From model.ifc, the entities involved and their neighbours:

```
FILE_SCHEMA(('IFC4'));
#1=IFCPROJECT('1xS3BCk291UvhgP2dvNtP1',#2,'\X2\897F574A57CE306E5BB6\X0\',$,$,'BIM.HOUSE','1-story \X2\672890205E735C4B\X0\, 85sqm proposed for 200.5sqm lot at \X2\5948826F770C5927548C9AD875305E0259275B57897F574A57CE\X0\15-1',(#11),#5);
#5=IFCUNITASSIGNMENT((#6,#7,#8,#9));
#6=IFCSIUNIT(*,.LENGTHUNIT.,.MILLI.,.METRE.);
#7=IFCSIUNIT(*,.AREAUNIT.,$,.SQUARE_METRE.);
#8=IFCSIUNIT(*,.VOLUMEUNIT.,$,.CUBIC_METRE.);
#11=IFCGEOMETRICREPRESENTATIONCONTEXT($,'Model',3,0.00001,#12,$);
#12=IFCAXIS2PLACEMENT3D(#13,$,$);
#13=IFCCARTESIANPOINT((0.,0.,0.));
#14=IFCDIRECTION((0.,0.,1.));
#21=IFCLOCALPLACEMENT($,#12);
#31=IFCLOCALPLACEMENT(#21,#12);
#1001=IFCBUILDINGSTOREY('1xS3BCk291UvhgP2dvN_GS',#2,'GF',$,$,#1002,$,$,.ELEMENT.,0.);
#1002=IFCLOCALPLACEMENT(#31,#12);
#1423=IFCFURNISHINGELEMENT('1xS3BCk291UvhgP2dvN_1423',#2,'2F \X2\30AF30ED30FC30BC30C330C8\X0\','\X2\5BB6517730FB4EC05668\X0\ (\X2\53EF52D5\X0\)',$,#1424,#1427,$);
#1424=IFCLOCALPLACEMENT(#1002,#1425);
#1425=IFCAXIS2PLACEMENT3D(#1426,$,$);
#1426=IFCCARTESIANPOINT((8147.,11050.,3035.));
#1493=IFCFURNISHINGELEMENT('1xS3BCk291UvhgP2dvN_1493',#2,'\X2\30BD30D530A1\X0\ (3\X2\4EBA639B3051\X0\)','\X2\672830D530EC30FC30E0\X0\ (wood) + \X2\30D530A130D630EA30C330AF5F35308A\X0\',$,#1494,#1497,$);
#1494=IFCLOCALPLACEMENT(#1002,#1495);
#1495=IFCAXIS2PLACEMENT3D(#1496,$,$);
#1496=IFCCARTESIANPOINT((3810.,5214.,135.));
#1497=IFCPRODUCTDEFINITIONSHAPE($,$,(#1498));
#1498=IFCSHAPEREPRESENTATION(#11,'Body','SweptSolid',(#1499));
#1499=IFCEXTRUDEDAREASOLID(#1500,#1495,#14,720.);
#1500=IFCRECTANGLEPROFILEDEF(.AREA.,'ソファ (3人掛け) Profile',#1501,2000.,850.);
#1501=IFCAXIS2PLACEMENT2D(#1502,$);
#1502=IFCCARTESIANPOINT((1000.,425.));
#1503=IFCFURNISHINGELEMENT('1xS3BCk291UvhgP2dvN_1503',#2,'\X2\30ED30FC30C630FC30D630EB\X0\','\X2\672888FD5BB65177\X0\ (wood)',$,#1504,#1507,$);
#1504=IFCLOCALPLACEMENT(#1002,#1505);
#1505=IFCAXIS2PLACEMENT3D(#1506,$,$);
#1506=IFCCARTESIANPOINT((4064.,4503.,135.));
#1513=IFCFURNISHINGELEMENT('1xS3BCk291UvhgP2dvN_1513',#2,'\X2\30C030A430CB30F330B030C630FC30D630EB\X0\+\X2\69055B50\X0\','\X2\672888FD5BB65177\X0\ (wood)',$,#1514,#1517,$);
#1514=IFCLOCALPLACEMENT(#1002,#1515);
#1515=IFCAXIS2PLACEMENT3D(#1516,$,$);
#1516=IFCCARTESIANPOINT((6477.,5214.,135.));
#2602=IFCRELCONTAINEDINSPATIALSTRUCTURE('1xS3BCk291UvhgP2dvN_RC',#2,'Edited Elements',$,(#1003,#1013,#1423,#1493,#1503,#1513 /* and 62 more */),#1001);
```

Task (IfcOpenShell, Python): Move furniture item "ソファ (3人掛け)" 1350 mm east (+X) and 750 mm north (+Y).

```python
import ifcopenshell
import ifcopenshell.api.geometry
import ifcopenshell.util.placement
import ifcopenshell.util.unit

model = ifcopenshell.open("model.ifc")
unit_scale = ifcopenshell.util.unit.calculate_unit_scale(model)

item = model.by_guid("1xS3BCk291UvhgP2dvN_1493")
matrix = ifcopenshell.util.placement.get_local_placement(item.ObjectPlacement)
matrix[0, 3] += 1.35 / unit_scale
matrix[1, 3] += 0.75 / unit_scale
ifcopenshell.api.geometry.edit_object_placement(model, product=item, matrix=matrix, is_si=False)

print(ifcopenshell.util.placement.get_local_placement(item.ObjectPlacement).round(3) + 0.0)

model.write("model_rev.ifc")
```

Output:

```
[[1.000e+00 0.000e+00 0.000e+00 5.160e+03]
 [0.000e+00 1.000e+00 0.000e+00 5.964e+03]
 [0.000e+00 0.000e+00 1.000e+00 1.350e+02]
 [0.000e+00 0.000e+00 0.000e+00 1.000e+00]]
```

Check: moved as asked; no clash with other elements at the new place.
